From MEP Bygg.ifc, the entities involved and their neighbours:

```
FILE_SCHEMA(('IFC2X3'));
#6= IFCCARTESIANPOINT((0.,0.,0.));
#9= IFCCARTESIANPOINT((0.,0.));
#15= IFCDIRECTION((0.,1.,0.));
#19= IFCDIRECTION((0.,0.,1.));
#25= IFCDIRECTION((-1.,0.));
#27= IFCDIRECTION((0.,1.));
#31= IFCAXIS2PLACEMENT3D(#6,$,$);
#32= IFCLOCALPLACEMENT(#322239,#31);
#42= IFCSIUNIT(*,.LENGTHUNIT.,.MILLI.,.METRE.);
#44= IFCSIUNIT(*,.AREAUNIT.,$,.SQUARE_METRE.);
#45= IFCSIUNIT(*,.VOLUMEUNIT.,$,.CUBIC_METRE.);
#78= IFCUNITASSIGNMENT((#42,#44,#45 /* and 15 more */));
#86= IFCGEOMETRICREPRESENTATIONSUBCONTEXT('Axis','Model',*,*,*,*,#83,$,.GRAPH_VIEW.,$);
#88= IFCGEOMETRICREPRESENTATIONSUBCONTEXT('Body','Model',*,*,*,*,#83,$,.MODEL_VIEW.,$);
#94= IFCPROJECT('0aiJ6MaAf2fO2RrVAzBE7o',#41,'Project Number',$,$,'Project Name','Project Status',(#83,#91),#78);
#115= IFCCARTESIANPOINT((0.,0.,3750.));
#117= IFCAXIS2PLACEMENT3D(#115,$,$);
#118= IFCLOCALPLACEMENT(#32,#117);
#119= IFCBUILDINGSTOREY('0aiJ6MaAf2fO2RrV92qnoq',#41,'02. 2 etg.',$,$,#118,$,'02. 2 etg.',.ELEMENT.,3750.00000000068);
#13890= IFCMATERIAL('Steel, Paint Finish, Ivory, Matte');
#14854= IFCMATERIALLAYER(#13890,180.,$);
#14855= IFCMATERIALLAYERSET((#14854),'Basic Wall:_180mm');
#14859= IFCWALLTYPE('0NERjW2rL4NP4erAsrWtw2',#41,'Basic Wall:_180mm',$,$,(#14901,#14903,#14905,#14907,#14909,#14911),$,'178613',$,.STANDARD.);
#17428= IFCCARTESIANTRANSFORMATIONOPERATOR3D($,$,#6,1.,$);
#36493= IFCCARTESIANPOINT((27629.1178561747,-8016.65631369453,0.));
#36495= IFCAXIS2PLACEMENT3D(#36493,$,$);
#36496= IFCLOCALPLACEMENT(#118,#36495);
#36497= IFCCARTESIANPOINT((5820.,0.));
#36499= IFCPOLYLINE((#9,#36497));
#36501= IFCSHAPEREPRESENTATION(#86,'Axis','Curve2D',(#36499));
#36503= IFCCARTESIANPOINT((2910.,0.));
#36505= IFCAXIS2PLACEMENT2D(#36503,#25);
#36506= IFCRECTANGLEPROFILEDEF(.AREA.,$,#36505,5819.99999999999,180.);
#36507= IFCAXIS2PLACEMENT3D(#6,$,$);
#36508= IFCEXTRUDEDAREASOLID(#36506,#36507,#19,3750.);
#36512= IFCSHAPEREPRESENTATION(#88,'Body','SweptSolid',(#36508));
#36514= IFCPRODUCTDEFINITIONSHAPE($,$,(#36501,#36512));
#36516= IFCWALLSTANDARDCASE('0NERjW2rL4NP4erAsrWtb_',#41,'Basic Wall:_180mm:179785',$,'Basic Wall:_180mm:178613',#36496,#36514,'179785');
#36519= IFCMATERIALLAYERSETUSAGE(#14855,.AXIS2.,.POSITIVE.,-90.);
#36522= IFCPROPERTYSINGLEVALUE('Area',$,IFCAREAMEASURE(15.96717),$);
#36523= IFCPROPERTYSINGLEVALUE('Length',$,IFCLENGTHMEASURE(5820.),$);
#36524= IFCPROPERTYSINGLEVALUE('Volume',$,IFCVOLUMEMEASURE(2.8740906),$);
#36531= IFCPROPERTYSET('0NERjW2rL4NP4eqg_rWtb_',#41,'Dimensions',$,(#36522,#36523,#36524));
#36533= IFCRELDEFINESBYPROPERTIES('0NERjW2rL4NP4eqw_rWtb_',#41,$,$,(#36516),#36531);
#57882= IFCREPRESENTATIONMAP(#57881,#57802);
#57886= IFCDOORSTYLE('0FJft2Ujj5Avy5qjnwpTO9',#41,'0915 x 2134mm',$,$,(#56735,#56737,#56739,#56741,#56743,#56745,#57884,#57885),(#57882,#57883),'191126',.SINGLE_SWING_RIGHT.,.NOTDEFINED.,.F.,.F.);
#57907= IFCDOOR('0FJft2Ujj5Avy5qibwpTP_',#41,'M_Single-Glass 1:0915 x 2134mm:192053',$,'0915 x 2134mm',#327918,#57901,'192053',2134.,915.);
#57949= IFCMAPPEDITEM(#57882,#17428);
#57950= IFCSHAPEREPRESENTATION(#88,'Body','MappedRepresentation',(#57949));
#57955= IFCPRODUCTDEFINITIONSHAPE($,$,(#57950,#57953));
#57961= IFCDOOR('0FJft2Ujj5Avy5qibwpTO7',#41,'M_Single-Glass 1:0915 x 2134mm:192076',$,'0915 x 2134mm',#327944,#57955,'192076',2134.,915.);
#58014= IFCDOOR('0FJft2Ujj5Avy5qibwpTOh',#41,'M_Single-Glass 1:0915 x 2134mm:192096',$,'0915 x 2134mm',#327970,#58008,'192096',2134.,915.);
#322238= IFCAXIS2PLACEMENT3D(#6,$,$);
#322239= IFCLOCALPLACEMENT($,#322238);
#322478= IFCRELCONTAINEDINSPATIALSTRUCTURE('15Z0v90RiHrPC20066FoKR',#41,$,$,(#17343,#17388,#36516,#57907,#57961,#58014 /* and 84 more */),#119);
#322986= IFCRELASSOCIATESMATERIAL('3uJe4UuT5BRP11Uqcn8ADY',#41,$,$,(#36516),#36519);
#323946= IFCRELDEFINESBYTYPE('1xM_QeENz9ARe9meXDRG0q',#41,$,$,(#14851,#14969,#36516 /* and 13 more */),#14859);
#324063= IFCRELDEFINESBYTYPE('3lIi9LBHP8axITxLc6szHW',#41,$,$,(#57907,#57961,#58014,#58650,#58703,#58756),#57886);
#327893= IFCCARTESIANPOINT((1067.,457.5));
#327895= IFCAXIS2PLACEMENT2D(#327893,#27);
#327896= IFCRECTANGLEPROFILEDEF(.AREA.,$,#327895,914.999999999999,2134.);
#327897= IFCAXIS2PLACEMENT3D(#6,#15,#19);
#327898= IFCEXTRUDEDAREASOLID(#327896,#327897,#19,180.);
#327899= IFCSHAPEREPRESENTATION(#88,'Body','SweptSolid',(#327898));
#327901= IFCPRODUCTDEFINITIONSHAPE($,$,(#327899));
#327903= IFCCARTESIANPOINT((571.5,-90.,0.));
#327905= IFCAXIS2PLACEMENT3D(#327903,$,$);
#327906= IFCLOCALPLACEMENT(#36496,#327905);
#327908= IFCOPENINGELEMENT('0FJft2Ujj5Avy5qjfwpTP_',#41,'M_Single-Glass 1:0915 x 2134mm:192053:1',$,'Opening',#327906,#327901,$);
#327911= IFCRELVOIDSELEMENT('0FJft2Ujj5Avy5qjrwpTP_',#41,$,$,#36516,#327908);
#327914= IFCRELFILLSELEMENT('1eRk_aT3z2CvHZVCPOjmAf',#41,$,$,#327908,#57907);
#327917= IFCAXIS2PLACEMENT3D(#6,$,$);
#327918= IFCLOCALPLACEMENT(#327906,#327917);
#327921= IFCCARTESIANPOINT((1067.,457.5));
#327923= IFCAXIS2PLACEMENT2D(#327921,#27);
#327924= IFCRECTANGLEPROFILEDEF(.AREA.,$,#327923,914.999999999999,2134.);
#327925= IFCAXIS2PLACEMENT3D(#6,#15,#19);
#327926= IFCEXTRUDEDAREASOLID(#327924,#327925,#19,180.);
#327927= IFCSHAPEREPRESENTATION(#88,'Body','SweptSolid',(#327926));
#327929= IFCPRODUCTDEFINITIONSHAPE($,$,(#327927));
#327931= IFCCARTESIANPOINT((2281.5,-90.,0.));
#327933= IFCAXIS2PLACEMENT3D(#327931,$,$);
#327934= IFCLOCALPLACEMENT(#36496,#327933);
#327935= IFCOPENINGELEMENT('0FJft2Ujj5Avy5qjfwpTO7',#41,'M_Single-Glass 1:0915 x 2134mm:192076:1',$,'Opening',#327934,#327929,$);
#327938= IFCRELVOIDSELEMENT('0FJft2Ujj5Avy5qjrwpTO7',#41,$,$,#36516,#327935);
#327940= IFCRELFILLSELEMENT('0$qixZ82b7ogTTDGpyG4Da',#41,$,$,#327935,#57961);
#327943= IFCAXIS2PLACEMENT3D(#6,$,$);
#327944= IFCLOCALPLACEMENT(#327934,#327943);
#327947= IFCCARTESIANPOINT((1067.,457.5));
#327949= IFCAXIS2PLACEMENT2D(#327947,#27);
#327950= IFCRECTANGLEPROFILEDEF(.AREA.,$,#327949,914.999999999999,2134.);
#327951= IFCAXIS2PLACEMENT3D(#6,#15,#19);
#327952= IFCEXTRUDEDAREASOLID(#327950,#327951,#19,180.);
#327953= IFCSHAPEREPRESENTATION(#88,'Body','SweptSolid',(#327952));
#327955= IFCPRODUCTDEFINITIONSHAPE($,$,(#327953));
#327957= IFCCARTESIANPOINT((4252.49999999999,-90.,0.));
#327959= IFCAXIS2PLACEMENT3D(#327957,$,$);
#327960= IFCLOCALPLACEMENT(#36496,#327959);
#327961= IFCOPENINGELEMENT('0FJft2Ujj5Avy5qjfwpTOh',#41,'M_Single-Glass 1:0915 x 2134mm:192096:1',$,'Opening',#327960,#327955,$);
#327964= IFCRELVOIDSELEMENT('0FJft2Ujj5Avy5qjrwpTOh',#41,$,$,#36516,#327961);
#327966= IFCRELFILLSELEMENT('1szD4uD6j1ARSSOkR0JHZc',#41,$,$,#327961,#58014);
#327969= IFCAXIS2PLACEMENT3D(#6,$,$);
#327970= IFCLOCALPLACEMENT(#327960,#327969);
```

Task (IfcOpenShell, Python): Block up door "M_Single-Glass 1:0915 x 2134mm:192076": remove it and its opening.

```python
import ifcopenshell
import ifcopenshell.api.feature
import ifcopenshell.api.pset
import ifcopenshell.api.root
import ifcopenshell.geom
import ifcopenshell.util.element
import ifcopenshell.util.shape
import ifcopenshell.util.unit

model = ifcopenshell.open("MEP Bygg.ifc")
area_scale = ifcopenshell.util.unit.calculate_unit_scale(model, "AREAUNIT")
volume_scale = ifcopenshell.util.unit.calculate_unit_scale(model, "VOLUMEUNIT")
settings = ifcopenshell.geom.settings()


def volume(element):
    """Net volume in cubic metres, openings subtracted."""
    shape = ifcopenshell.geom.create_shape(settings, element)
    return ifcopenshell.util.shape.get_volume(shape.geometry)


door = model.by_guid("0FJft2Ujj5Avy5qibwpTO7")
opening = door.FillsVoids[0].RelatingOpeningElement
wall = opening.VoidsElements[0].RelatingBuildingElement
before = volume(wall)

ifcopenshell.api.root.remove_product(model, product=door)
ifcopenshell.api.feature.remove_feature(model, feature=opening)

after = volume(wall)
thickness = 0.18  # wall thickness in metres

# Update the wall's stored quantities.
pset = model.by_id(ifcopenshell.util.element.get_pset(wall, "Dimensions", should_inherit=False)["id"])
ifcopenshell.api.pset.edit_pset(model, pset=pset, properties={
    "Area": model.create_entity("IfcAreaMeasure", after / thickness / area_scale),
    "Volume": model.create_entity("IfcVolumeMeasure", after / volume_scale),
})

print(f"wall volume {before:.3f} -> {after:.3f} m3")

model.write("MEP Bygg_updated.ifc")
```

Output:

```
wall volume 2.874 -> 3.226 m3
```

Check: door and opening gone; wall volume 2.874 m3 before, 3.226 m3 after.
